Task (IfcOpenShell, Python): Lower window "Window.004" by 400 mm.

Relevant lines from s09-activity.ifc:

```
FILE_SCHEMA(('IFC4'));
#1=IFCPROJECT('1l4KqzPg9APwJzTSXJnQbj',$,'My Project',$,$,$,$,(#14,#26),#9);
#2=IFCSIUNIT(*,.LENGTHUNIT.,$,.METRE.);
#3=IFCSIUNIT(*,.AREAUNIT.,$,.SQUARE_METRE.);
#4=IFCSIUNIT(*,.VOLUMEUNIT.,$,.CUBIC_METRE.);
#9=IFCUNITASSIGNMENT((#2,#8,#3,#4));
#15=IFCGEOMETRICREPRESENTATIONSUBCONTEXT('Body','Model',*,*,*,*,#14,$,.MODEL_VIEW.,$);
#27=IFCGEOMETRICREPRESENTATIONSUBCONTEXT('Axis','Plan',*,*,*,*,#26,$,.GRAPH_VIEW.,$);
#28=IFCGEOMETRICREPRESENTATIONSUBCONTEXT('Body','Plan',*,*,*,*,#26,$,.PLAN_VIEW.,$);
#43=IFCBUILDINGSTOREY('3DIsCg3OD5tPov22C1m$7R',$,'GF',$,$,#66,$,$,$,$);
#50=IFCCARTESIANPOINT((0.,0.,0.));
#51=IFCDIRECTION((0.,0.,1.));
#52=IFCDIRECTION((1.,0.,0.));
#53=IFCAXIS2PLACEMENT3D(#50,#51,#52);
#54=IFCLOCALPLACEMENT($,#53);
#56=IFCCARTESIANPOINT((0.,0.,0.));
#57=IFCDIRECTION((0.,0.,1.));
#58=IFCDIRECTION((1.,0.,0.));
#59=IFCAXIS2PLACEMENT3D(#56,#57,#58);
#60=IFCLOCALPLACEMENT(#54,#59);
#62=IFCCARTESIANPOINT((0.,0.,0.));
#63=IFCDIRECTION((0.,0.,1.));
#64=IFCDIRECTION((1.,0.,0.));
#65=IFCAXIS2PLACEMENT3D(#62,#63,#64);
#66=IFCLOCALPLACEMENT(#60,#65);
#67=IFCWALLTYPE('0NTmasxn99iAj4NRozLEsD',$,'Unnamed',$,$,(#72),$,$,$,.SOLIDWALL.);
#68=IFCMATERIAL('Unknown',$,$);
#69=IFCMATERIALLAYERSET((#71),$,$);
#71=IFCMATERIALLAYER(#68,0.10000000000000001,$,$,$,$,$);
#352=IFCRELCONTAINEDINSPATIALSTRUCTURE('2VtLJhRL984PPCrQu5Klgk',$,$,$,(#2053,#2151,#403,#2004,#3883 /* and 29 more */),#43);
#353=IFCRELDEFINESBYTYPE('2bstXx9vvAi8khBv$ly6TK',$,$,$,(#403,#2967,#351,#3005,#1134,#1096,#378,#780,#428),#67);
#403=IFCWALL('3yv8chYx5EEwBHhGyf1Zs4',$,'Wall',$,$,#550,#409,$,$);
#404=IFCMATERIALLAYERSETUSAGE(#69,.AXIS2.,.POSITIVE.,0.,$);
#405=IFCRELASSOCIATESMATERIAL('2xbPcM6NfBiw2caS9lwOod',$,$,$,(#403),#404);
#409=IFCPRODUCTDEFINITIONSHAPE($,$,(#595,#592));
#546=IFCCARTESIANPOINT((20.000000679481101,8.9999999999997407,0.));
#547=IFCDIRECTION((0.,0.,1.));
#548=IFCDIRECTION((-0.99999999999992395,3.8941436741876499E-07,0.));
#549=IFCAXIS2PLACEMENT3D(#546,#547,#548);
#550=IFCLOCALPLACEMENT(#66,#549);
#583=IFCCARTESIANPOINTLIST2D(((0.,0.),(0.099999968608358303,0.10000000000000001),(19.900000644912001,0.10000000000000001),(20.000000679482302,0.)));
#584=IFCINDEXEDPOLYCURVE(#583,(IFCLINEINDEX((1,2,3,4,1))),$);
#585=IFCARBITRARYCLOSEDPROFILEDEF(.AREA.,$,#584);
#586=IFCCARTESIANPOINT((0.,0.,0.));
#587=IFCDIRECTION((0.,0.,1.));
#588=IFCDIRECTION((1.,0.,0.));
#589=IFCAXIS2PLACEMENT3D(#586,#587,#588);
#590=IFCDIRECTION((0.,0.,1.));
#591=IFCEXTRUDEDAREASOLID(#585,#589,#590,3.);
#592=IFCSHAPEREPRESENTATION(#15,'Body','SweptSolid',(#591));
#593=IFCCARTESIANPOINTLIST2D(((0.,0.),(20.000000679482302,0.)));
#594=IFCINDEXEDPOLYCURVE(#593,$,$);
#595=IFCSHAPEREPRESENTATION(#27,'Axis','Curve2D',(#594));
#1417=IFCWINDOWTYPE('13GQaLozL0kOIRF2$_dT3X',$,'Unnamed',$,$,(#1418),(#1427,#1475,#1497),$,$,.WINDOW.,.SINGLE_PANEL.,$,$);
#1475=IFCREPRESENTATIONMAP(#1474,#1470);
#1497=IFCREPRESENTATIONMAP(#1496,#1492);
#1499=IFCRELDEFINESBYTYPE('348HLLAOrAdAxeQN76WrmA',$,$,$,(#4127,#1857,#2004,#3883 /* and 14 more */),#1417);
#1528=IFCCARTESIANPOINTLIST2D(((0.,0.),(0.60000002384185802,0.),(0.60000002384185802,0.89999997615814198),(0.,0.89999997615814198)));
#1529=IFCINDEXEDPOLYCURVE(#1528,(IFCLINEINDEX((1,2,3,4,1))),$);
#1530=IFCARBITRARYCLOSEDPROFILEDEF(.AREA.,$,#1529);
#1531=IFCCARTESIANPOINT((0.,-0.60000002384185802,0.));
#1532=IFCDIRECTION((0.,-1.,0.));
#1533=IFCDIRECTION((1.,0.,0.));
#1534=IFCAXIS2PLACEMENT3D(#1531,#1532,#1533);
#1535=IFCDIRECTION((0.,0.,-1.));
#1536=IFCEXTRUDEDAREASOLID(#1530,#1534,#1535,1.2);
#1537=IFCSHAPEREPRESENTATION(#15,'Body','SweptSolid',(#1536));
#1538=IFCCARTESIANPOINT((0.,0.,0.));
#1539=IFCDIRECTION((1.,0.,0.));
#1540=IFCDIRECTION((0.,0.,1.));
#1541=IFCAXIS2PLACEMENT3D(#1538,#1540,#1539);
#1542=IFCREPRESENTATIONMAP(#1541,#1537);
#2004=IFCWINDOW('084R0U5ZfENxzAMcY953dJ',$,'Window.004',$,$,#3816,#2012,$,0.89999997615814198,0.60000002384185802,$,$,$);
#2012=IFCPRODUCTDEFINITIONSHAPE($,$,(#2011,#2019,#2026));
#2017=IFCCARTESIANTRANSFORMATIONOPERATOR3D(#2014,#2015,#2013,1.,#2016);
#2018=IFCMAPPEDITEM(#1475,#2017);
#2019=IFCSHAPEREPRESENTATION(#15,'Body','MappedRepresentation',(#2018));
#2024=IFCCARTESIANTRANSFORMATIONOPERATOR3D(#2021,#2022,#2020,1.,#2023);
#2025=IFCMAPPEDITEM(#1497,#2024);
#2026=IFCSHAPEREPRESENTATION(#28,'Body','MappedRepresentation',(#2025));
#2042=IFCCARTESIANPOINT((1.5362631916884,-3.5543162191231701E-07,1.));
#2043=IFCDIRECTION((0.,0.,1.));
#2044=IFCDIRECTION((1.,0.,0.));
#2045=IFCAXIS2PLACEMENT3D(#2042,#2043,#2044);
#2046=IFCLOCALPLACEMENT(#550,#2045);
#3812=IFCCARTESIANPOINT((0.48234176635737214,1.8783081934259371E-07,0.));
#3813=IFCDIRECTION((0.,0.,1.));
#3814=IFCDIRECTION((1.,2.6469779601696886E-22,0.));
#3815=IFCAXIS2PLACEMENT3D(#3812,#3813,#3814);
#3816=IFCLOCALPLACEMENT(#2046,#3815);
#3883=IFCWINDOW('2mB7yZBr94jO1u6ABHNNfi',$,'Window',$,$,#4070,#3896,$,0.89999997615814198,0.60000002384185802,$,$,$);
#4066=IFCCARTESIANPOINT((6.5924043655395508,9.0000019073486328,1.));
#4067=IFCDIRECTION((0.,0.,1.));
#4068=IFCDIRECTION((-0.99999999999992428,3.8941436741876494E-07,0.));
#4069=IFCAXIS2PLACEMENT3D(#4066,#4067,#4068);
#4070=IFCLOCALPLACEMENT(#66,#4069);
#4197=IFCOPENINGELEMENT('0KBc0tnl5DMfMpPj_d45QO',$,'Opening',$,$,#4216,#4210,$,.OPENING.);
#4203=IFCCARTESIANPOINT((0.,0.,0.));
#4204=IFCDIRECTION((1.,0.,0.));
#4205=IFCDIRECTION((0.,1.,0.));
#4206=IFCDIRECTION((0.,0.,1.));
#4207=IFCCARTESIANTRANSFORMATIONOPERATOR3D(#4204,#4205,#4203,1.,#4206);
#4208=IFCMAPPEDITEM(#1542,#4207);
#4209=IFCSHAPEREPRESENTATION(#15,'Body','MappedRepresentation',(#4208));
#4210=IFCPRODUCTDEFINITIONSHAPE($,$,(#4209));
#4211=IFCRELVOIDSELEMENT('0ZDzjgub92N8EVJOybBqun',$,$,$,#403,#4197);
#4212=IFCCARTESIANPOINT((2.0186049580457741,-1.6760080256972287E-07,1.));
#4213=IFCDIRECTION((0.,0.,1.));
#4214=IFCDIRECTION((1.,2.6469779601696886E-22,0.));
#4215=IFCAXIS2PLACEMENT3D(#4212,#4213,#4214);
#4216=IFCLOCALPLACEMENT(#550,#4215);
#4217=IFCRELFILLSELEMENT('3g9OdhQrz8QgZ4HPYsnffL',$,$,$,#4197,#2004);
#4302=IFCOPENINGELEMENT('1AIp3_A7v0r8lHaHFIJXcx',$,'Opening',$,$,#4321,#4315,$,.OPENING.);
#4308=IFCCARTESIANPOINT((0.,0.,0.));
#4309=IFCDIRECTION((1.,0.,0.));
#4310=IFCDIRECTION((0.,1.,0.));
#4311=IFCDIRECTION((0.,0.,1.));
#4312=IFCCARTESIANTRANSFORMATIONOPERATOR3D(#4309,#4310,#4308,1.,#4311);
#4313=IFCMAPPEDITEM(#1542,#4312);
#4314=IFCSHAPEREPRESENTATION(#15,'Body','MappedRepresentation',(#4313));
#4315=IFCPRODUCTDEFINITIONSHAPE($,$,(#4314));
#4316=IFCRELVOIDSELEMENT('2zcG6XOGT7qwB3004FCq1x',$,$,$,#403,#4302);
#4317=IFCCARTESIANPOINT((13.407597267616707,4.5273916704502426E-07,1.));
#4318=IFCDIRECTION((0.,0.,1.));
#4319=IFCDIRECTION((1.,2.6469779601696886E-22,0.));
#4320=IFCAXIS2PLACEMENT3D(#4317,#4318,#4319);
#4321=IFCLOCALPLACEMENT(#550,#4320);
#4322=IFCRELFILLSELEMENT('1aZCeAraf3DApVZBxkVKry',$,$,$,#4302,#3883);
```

```python
import numpy as np
import ifcopenshell
import ifcopenshell.api.geometry
import ifcopenshell.util.placement
import ifcopenshell.util.unit

model = ifcopenshell.open("s09-activity.ifc")
unit_scale = ifcopenshell.util.unit.calculate_unit_scale(model)

window = model.by_guid("084R0U5ZfENxzAMcY953dJ")
opening = window.FillsVoids[0].RelatingOpeningElement
dz = -0.4

shift = np.array([0.0, 0.0, dz])
# The window is not placed relative to its opening, so move both.
for product in (opening, window):
    matrix = ifcopenshell.util.placement.get_local_placement(product.ObjectPlacement)
    matrix[:3, 3] += shift
    ifcopenshell.api.geometry.edit_object_placement(model, product=product, matrix=matrix, is_si=False)

print(f"moved by {dz * unit_scale:+.3f} m")

model.write("s09-activity_v2.ifc")
```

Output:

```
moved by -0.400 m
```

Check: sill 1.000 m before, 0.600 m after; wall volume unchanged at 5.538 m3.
